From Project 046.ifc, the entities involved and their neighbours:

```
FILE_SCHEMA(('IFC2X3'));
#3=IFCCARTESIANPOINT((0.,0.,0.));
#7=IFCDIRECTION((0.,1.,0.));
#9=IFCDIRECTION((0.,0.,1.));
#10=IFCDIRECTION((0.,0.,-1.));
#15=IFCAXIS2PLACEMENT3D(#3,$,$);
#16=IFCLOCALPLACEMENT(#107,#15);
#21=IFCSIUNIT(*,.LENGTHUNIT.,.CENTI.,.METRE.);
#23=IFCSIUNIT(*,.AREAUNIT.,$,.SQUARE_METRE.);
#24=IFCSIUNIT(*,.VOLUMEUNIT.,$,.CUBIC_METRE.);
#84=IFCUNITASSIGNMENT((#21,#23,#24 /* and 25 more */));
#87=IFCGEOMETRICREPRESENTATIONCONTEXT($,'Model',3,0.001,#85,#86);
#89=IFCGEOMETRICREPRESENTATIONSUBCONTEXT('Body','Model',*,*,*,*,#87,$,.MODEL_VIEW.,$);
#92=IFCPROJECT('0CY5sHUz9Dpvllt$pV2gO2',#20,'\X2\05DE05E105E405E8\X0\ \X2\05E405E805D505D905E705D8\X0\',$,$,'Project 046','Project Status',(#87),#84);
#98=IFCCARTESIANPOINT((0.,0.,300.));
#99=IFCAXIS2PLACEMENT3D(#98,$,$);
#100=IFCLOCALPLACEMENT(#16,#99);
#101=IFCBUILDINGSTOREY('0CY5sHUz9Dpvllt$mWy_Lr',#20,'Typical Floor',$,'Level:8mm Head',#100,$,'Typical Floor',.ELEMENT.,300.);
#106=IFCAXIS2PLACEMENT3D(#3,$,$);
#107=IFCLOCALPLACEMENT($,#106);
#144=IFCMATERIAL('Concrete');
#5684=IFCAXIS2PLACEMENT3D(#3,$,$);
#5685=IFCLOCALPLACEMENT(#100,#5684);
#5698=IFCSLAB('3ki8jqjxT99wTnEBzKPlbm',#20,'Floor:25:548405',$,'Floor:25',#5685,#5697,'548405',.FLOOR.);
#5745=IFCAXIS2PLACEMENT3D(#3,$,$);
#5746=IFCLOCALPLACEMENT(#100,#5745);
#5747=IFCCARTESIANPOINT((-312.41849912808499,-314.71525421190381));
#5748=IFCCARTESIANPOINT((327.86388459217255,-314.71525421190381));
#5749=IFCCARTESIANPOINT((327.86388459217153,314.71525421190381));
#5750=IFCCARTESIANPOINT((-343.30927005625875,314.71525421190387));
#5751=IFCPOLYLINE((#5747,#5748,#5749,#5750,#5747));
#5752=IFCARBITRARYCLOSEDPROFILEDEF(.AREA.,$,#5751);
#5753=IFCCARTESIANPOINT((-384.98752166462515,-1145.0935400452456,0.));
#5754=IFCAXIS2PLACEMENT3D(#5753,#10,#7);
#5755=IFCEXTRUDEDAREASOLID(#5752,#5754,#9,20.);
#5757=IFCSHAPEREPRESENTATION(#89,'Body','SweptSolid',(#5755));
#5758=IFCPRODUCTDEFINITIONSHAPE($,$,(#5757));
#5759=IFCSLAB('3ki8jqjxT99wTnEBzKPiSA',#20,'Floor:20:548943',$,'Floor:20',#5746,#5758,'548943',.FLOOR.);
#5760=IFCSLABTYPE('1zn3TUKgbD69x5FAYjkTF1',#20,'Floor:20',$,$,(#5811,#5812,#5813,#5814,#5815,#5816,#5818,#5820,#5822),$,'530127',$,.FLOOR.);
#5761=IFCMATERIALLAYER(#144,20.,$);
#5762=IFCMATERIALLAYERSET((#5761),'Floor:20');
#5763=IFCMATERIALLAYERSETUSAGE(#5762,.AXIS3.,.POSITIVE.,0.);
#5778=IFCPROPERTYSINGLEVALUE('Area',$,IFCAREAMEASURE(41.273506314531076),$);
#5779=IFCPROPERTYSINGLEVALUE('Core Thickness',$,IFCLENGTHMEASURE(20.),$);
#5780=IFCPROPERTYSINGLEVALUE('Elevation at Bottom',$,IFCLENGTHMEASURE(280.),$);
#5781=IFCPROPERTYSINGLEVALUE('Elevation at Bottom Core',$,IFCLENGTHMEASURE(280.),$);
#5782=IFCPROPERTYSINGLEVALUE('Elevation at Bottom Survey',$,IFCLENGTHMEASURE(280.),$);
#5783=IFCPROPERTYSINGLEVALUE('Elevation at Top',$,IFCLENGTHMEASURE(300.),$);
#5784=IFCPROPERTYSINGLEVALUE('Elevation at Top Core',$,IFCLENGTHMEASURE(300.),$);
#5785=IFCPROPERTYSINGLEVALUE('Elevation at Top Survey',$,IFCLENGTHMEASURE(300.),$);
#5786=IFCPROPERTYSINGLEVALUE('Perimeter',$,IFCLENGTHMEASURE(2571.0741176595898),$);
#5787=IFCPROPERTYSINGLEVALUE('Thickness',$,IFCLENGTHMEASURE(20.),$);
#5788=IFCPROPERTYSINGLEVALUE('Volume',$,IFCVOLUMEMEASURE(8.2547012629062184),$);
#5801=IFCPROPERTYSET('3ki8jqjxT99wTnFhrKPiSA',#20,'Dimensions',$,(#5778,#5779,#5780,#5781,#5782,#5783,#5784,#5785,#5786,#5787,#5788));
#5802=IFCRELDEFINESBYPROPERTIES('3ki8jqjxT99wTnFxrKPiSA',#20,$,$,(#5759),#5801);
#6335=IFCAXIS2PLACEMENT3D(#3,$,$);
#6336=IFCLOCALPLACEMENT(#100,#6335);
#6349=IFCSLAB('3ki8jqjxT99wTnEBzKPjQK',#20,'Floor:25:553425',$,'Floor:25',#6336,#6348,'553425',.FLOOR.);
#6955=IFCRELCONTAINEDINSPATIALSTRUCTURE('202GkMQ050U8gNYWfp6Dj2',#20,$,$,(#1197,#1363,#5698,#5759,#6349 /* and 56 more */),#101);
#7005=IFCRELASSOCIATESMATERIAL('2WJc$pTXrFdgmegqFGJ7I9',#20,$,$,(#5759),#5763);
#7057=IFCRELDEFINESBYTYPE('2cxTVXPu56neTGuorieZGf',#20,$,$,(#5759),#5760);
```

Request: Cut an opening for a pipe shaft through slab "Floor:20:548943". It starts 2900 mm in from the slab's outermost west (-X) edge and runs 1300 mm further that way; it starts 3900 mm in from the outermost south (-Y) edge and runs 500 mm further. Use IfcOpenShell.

```python
import numpy as np
import ifcopenshell
import ifcopenshell.api.feature
import ifcopenshell.api.geometry
import ifcopenshell.api.pset
import ifcopenshell.api.root
import ifcopenshell.geom
import ifcopenshell.util.element
import ifcopenshell.util.placement
import ifcopenshell.util.representation
import ifcopenshell.util.shape
import ifcopenshell.util.unit

model = ifcopenshell.open("Project 046.ifc")
unit_scale = ifcopenshell.util.unit.calculate_unit_scale(model)
area_scale = ifcopenshell.util.unit.calculate_unit_scale(model, "AREAUNIT")
volume_scale = ifcopenshell.util.unit.calculate_unit_scale(model, "VOLUMEUNIT")
settings = ifcopenshell.geom.settings()


def volume(element):
    """Net volume in cubic metres, openings subtracted."""
    shape = ifcopenshell.geom.create_shape(settings, element)
    return ifcopenshell.util.shape.get_volume(shape.geometry)


slab = model.by_guid("3ki8jqjxT99wTnEBzKPiSA")
before = volume(slab)

# Extent in the slab's own axes, in metres. The edges named are its -X and -Y sides.
slab_shape = ifcopenshell.geom.create_shape(settings, slab)
vertices = ifcopenshell.util.shape.get_vertices(slab_shape.geometry)
x_min, y_min, bottom = vertices.min(axis=0)
top = vertices[:, 2].max()

opening = ifcopenshell.api.root.create_entity(model, ifc_class="IfcOpeningElement", name="Pipe shaft opening")
context = ifcopenshell.util.representation.get_context(model, "Model", "Body", "MODEL_VIEW")
width, depth = 1.3, 0.5
outline = [(0.0, 0.0), (width, 0.0), (width, depth), (0.0, depth), (0.0, 0.0)]
# Overshoot both faces by 50 mm so the cut is clean.
shape = ifcopenshell.api.geometry.add_slab_representation(
    model, context=context, depth=top - bottom + 0.1, polyline=outline
)
ifcopenshell.api.geometry.assign_representation(model, product=opening, representation=shape)

matrix = ifcopenshell.util.placement.get_local_placement(slab.ObjectPlacement)
matrix[:, 3] = matrix @ np.append(np.array([x_min + 2.9, y_min + 3.9, bottom - 0.05]) / unit_scale, 1.0)
ifcopenshell.api.geometry.edit_object_placement(model, product=opening, matrix=matrix, is_si=False)
ifcopenshell.api.feature.add_feature(model, feature=opening, element=slab)

after = volume(slab)

# Update the slab's stored quantities.
pset = model.by_id(ifcopenshell.util.element.get_pset(slab, "Dimensions", should_inherit=False)["id"])
ifcopenshell.api.pset.edit_pset(model, pset=pset, properties={
    "Area": model.create_entity("IfcAreaMeasure", after / (top - bottom) / area_scale),
    "Volume": model.create_entity("IfcVolumeMeasure", after / volume_scale),
})

print(f"slab volume {before:.3f} -> {after:.3f} m3")

model.write("Project 046_edited.ifc")
```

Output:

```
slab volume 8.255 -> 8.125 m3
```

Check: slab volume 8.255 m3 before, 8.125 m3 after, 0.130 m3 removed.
